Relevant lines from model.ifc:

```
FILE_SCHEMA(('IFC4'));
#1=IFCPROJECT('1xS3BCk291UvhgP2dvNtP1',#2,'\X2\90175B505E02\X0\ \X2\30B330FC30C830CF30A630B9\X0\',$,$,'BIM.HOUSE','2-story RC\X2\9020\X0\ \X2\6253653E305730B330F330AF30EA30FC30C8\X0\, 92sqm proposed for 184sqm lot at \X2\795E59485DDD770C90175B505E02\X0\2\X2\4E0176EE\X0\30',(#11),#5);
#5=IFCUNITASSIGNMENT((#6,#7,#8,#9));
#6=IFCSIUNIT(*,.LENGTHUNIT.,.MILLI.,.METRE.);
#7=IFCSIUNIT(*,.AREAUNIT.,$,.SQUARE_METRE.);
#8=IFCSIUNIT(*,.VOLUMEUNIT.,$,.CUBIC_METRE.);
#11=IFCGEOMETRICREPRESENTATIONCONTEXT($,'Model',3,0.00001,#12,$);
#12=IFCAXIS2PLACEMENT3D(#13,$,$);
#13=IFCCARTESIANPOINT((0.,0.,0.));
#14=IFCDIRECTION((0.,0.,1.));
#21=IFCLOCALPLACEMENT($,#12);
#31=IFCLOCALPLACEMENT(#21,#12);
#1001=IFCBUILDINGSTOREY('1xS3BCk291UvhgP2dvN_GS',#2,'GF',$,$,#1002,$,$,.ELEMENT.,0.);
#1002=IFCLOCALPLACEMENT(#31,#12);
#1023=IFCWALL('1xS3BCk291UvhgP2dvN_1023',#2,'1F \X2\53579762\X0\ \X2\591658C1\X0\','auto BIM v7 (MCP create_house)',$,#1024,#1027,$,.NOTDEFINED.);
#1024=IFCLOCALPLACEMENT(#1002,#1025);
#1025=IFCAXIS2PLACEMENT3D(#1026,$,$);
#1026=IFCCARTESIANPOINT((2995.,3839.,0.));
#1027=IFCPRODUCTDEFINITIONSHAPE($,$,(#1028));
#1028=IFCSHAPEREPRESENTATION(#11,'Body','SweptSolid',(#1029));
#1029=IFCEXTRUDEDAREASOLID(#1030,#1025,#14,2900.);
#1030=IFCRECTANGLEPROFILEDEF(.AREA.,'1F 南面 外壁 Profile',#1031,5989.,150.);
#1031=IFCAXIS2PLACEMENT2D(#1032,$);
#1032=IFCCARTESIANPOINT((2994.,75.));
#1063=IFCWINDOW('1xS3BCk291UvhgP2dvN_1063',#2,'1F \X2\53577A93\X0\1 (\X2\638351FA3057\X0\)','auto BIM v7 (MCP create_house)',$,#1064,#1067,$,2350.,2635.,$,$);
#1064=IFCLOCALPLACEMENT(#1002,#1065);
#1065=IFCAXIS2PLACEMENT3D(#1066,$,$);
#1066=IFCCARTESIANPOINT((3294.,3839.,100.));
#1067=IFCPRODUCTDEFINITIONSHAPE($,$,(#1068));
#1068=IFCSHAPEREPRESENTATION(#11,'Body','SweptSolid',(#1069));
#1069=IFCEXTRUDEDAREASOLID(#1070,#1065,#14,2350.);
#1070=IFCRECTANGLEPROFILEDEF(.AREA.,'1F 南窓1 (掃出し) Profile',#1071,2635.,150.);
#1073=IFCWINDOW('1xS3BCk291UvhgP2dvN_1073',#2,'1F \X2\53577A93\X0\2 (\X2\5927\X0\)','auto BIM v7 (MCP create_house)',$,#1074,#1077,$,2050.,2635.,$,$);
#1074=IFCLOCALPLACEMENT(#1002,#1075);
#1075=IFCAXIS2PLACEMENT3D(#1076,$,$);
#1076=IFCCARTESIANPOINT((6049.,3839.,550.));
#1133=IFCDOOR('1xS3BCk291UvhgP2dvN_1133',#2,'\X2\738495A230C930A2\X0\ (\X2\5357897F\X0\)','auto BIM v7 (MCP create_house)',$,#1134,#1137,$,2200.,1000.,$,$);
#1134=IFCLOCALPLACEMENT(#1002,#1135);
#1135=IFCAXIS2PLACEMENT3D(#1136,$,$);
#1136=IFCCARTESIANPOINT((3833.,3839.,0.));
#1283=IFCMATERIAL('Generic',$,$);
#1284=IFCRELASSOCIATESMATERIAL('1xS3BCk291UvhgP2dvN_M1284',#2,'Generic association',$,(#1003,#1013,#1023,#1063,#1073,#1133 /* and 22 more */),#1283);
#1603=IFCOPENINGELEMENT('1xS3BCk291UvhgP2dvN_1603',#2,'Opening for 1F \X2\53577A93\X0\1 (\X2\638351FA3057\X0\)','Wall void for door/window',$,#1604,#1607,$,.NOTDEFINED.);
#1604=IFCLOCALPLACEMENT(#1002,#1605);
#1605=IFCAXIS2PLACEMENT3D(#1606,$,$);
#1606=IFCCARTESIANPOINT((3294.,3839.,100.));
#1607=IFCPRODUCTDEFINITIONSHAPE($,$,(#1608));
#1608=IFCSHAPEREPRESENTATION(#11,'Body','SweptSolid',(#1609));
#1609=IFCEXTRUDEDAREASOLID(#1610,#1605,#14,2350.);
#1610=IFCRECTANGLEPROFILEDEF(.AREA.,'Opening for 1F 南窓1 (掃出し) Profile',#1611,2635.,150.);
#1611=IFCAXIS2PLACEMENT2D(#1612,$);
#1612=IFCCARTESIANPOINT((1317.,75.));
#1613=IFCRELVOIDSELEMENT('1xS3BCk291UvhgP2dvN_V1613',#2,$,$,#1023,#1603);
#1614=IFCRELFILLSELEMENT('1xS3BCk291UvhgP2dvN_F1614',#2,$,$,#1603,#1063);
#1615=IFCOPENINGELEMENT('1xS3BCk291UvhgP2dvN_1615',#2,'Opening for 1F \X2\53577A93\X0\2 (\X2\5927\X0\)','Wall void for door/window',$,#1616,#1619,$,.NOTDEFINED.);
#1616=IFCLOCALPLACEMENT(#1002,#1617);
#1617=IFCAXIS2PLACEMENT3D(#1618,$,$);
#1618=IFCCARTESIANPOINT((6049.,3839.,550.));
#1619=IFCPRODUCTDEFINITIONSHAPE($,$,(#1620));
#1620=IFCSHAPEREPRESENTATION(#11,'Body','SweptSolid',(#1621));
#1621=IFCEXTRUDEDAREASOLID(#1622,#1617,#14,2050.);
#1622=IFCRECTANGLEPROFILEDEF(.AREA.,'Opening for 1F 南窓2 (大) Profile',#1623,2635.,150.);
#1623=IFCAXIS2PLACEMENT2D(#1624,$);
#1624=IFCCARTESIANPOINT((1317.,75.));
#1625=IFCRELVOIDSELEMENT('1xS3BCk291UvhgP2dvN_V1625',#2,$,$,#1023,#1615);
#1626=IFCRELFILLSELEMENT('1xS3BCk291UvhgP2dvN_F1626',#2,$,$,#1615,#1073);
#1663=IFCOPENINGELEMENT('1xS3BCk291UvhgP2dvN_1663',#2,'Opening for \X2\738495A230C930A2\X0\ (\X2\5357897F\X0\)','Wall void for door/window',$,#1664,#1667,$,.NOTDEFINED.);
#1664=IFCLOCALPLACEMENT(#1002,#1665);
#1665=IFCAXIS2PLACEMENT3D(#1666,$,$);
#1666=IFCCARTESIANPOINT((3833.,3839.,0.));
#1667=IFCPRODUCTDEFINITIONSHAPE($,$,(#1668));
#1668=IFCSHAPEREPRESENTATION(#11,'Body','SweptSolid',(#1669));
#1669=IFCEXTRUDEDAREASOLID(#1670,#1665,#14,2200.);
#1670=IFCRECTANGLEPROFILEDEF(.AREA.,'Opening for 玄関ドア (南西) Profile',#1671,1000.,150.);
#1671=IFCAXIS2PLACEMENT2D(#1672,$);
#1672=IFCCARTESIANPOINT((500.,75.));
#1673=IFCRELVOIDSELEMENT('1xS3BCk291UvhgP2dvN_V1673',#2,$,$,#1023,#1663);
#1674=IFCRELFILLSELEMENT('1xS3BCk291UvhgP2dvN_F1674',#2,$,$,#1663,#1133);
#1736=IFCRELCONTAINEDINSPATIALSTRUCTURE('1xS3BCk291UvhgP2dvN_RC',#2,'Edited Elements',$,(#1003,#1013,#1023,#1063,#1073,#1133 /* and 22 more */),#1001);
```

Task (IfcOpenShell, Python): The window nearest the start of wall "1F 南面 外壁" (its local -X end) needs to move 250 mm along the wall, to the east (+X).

```python
import ifcopenshell
import ifcopenshell.api.geometry
import ifcopenshell.util.placement
import ifcopenshell.util.unit

model = ifcopenshell.open("model.ifc")
unit_scale = ifcopenshell.util.unit.calculate_unit_scale(model)

window = model.by_id(1063)
opening = window.FillsVoids[0].RelatingOpeningElement
wall = opening.VoidsElements[0].RelatingBuildingElement

wall_matrix = ifcopenshell.util.placement.get_local_placement(wall.ObjectPlacement)
shift = wall_matrix[:3, 0] * 0.25 / unit_scale
before = ifcopenshell.util.placement.get_local_placement(window.ObjectPlacement)[:3, 3].copy()

# The window is not placed relative to its opening, so move both.
for product in (opening, window):
    matrix = ifcopenshell.util.placement.get_local_placement(product.ObjectPlacement)
    matrix[:3, 3] += shift
    ifcopenshell.api.geometry.edit_object_placement(model, product=product, matrix=matrix, is_si=False)

after = ifcopenshell.util.placement.get_local_placement(window.ObjectPlacement)[:3, 3]
print("window moved by", (after - before).round(3) + 0.0)

model.write("model_updated.ifc")
```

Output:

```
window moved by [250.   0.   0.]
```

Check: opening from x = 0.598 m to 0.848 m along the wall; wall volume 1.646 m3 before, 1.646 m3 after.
